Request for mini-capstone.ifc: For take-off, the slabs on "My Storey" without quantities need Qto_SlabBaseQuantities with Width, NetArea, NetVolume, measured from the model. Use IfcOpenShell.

First a look at what the model holds.

```python
import ifcopenshell
import ifcopenshell.util.element
import ifcopenshell.util.unit

model = ifcopenshell.open("mini-capstone.ifc")
print(model.schema)
for unit_type in ("LENGTHUNIT", "AREAUNIT", "VOLUMEUNIT"):
    print(unit_type, ifcopenshell.util.unit.calculate_unit_scale(model, unit_type))
storey = next(s for s in model.by_type("IfcBuildingStorey") if s.Name == "My Storey")
slabs = [e for e in ifcopenshell.util.element.get_decomposition(storey) if e.is_a("IfcSlab")]
for e in sorted(slabs, key=lambda e: e.id()):
    print(e.id(), e.is_a(), e.Name, list(ifcopenshell.util.element.get_psets(e, qtos_only=True)), sep=" | ")
```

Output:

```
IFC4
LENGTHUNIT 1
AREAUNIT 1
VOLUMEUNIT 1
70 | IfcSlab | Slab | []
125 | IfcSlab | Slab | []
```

```python
import ifcopenshell
import ifcopenshell.api.pset
import ifcopenshell.geom
import ifcopenshell.util.element
import ifcopenshell.util.shape
import ifcopenshell.util.unit

model = ifcopenshell.open("mini-capstone.ifc")
unit_scale = ifcopenshell.util.unit.calculate_unit_scale(model)
area_scale = ifcopenshell.util.unit.calculate_unit_scale(model, "AREAUNIT")
volume_scale = ifcopenshell.util.unit.calculate_unit_scale(model, "VOLUMEUNIT")
settings = ifcopenshell.geom.settings()

storey = next(s for s in model.by_type("IfcBuildingStorey") if s.Name == "My Storey")
slabs = [e for e in ifcopenshell.util.element.get_decomposition(storey) if e.is_a("IfcSlab")]

for e in sorted(slabs, key=lambda e: e.id()):
    if ifcopenshell.util.element.get_psets(e, qtos_only=True, should_inherit=False):
        continue
    # Geometry comes back in metres, in the element's own axes.
    shape = ifcopenshell.geom.create_shape(settings, e)
    values = {
        "Width": ifcopenshell.util.shape.get_z(shape.geometry) / unit_scale,
        "NetArea": ifcopenshell.util.shape.get_footprint_area(shape.geometry) / area_scale,
        "NetVolume": ifcopenshell.util.shape.get_volume(shape.geometry) / volume_scale,
    }
    qto = ifcopenshell.api.pset.add_qto(model, product=e, name="Qto_SlabBaseQuantities")
    ifcopenshell.api.pset.edit_qto(model, qto=qto, properties=values)
    print(e.id(), {k: round(v, 3) for k, v in values.items()})

model.write("mini-capstone_v2.ifc")
```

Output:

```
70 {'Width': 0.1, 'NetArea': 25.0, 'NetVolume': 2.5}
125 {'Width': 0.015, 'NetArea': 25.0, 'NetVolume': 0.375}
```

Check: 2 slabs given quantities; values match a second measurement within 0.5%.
